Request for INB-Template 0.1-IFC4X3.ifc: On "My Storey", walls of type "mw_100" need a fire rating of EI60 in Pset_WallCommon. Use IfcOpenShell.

First a look at what the model holds.

```python
import ifcopenshell
import ifcopenshell.util.element

model = ifcopenshell.open("INB-Template 0.1-IFC4X3.ifc")
print(model.schema)
storey = next(s for s in model.by_type("IfcBuildingStorey") if s.Name == "My Storey")
walls = [e for e in ifcopenshell.util.element.get_decomposition(storey) if e.is_a("IfcWall")]
seen = {}
for e in walls:
    element_type = ifcopenshell.util.element.get_type(e)
    key = (element_type.Name if element_type != e and element_type else None, ifcopenshell.util.element.get_pset(e, "Pset_WallCommon", "FireRating"))
    seen[key] = seen.get(key, 0) + 1
for (name, value), count in sorted(seen.items(), key=str):
    print(count, "x", name, "|", value)
```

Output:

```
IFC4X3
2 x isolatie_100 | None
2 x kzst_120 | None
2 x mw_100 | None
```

```python
import ifcopenshell
import ifcopenshell.api.pset
import ifcopenshell.util.element

model = ifcopenshell.open("INB-Template 0.1-IFC4X3.ifc")

storey = next(s for s in model.by_type("IfcBuildingStorey") if s.Name == "My Storey")
walls = [e for e in ifcopenshell.util.element.get_decomposition(storey) if e.is_a("IfcWall")]

count = 0
for e in walls:
    element_type = ifcopenshell.util.element.get_type(e)
    if element_type in (None, e) or element_type.Name != "mw_100":
        continue
    # add_pset returns the element's existing set when there is one.
    pset = ifcopenshell.api.pset.add_pset(model, product=e, name="Pset_WallCommon")
    ifcopenshell.api.pset.edit_pset(model, pset=pset, properties={"FireRating": "EI60"})
    count += 1

print(count, "walls updated")

model.write("INB-Template 0.1-IFC4X3_v2.ifc")
```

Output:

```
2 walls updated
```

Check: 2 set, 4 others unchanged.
